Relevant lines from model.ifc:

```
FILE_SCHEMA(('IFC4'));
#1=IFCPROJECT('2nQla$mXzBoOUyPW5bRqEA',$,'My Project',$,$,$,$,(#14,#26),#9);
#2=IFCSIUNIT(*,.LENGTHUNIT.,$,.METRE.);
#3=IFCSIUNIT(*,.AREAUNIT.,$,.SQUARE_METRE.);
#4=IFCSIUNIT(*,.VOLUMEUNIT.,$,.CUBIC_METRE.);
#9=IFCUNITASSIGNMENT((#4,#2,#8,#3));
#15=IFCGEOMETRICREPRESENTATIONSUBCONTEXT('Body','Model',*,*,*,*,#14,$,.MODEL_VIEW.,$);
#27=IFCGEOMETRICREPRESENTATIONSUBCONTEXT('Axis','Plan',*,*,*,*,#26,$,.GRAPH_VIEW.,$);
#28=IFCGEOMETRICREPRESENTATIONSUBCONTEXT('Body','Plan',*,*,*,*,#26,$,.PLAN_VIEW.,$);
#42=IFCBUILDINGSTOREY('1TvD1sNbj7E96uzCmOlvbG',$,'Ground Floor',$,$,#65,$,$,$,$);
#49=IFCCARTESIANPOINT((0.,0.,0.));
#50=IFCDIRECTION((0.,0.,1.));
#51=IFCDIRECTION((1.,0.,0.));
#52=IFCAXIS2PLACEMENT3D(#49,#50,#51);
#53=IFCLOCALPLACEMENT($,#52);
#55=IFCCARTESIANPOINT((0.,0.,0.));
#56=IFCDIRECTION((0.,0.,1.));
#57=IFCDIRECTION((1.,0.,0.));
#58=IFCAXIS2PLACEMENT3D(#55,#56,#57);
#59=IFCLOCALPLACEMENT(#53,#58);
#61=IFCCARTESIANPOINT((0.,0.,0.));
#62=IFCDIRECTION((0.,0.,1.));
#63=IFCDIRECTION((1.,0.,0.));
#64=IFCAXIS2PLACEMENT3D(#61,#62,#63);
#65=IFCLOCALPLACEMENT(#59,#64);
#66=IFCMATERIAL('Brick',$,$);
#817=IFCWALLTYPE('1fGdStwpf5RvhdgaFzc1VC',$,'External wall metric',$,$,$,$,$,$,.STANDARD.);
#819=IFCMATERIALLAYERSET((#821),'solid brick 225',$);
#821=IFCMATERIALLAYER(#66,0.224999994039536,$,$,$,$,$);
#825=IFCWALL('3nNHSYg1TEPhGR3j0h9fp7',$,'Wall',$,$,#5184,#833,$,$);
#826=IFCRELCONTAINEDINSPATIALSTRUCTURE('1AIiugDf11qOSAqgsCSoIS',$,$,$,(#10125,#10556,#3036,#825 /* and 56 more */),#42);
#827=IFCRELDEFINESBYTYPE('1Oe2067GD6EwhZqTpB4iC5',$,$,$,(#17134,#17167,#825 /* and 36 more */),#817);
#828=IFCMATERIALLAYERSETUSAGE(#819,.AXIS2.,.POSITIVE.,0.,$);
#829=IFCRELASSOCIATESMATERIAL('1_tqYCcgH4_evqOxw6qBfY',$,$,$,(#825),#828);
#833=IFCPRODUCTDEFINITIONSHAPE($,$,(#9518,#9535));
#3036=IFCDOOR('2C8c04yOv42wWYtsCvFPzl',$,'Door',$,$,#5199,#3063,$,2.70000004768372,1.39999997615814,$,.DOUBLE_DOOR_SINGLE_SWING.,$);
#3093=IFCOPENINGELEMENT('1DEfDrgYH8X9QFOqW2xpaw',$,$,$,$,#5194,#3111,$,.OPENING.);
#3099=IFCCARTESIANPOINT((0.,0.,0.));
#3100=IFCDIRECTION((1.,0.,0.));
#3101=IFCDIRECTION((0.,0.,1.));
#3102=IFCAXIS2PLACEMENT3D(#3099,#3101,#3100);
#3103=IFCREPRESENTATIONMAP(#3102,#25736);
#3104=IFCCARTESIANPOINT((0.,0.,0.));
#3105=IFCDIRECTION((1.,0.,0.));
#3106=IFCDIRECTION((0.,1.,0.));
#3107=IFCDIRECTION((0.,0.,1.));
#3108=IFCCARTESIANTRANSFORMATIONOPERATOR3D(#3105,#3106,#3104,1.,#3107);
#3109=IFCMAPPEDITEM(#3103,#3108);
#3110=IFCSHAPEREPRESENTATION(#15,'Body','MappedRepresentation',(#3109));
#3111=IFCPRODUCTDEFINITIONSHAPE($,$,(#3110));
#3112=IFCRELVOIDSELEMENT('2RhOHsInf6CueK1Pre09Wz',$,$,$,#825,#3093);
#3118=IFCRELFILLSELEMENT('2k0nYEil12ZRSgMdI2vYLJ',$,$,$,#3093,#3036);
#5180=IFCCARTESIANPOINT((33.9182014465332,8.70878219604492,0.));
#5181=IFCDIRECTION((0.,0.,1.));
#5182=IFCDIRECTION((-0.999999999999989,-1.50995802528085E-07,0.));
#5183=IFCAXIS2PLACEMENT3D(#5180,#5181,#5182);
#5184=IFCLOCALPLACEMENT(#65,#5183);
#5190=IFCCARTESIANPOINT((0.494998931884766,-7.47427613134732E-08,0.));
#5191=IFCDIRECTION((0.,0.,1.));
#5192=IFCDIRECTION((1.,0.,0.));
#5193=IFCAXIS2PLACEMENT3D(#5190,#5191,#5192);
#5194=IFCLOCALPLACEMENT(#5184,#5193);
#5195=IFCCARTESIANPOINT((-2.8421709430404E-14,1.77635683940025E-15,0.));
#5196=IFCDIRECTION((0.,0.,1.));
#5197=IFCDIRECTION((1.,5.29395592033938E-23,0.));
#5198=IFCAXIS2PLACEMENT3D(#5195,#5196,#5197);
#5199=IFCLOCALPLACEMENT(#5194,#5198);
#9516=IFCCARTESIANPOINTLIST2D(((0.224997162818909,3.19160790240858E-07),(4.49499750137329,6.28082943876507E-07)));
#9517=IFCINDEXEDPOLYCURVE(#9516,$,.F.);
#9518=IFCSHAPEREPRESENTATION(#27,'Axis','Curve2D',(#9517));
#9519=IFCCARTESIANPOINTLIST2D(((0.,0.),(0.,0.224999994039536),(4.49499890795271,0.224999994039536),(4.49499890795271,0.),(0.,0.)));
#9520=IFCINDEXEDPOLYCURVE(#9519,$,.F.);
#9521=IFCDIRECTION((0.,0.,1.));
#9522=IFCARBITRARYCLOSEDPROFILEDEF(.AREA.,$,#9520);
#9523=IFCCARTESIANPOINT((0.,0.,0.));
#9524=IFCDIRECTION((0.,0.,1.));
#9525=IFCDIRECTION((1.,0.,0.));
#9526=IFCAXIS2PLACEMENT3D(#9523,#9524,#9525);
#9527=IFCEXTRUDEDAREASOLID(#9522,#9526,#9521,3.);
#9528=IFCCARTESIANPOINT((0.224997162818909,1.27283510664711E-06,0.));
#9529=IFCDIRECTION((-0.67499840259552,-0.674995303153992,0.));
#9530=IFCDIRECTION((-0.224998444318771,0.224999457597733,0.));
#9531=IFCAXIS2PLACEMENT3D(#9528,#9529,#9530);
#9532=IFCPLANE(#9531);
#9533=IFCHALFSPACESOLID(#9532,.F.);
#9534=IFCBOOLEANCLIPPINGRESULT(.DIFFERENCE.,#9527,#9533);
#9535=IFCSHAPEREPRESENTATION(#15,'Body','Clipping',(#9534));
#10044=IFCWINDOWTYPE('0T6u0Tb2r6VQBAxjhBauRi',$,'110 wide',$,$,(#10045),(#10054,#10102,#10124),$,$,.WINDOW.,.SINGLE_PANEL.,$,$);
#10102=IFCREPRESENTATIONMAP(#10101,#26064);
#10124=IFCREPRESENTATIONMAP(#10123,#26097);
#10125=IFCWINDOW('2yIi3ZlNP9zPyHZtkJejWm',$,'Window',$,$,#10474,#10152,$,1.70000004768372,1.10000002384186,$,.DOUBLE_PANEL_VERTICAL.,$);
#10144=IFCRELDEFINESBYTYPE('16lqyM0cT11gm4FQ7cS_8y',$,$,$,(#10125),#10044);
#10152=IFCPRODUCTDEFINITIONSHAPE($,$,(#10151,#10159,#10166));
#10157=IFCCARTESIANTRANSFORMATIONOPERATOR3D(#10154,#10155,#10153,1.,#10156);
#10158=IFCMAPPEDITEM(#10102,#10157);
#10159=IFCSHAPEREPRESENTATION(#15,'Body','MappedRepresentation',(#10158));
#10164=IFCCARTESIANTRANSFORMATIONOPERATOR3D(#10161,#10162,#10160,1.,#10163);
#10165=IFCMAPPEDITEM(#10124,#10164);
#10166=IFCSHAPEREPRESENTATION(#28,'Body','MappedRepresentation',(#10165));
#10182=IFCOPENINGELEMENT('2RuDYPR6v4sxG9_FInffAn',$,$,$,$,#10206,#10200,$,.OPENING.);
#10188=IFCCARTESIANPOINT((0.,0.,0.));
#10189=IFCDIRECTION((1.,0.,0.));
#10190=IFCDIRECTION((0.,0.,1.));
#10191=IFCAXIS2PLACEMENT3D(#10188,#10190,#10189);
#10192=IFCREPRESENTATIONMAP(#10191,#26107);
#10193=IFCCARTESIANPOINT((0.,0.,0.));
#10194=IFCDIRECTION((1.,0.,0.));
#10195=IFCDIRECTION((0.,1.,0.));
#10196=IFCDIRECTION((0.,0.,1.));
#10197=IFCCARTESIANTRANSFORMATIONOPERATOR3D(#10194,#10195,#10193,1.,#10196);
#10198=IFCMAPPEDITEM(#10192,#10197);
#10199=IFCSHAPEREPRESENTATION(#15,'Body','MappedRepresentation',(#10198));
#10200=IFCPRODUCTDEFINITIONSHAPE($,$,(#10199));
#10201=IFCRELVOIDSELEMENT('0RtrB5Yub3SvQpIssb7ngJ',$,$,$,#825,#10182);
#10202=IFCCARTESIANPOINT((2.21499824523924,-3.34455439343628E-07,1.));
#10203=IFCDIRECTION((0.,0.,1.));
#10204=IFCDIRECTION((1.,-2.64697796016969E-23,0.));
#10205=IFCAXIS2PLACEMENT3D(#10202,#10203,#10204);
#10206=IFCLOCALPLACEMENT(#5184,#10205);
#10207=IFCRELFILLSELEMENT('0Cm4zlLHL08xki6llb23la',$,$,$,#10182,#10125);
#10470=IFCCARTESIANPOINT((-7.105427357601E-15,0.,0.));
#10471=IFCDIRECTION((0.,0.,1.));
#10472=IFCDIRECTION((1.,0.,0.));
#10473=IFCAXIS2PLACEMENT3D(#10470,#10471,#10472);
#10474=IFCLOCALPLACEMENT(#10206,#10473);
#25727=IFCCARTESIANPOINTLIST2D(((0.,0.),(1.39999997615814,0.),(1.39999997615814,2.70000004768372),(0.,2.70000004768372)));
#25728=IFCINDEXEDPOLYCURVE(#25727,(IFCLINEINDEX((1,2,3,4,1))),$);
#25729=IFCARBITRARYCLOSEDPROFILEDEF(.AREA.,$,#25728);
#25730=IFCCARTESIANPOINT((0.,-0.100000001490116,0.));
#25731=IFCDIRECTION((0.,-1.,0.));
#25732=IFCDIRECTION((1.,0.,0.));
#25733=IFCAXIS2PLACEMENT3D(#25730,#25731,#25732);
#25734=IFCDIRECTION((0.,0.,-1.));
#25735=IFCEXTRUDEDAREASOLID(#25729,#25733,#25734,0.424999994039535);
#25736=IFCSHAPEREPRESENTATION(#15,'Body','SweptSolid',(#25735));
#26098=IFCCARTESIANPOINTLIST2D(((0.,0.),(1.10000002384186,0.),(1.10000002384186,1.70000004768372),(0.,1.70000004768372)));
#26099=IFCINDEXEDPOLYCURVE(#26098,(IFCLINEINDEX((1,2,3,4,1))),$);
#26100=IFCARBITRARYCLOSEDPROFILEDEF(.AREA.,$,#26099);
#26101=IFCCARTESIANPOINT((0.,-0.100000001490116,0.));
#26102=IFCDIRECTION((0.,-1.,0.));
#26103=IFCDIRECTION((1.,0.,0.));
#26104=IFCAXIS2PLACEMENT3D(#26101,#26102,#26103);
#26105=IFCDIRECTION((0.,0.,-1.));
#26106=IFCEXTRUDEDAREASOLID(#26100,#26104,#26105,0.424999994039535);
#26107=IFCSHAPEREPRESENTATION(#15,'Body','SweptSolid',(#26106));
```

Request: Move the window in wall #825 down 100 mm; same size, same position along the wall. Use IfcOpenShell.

```python
import numpy as np
import ifcopenshell
import ifcopenshell.api.geometry
import ifcopenshell.util.placement
import ifcopenshell.util.unit

model = ifcopenshell.open("model.ifc")
unit_scale = ifcopenshell.util.unit.calculate_unit_scale(model)

window = model.by_guid("2yIi3ZlNP9zPyHZtkJejWm")
opening = window.FillsVoids[0].RelatingOpeningElement
dz = -0.1

shift = np.array([0.0, 0.0, dz])
# The window is placed relative to its opening, so it follows when the opening moves.
matrix = ifcopenshell.util.placement.get_local_placement(opening.ObjectPlacement)
matrix[:3, 3] += shift
ifcopenshell.api.geometry.edit_object_placement(
    model, product=opening, matrix=matrix, is_si=False, should_transform_children=True
)

print(f"moved by {dz * unit_scale:+.3f} m")

model.write("model_updated.ifc")
```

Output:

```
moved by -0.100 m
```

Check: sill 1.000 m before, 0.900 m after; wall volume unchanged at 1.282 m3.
